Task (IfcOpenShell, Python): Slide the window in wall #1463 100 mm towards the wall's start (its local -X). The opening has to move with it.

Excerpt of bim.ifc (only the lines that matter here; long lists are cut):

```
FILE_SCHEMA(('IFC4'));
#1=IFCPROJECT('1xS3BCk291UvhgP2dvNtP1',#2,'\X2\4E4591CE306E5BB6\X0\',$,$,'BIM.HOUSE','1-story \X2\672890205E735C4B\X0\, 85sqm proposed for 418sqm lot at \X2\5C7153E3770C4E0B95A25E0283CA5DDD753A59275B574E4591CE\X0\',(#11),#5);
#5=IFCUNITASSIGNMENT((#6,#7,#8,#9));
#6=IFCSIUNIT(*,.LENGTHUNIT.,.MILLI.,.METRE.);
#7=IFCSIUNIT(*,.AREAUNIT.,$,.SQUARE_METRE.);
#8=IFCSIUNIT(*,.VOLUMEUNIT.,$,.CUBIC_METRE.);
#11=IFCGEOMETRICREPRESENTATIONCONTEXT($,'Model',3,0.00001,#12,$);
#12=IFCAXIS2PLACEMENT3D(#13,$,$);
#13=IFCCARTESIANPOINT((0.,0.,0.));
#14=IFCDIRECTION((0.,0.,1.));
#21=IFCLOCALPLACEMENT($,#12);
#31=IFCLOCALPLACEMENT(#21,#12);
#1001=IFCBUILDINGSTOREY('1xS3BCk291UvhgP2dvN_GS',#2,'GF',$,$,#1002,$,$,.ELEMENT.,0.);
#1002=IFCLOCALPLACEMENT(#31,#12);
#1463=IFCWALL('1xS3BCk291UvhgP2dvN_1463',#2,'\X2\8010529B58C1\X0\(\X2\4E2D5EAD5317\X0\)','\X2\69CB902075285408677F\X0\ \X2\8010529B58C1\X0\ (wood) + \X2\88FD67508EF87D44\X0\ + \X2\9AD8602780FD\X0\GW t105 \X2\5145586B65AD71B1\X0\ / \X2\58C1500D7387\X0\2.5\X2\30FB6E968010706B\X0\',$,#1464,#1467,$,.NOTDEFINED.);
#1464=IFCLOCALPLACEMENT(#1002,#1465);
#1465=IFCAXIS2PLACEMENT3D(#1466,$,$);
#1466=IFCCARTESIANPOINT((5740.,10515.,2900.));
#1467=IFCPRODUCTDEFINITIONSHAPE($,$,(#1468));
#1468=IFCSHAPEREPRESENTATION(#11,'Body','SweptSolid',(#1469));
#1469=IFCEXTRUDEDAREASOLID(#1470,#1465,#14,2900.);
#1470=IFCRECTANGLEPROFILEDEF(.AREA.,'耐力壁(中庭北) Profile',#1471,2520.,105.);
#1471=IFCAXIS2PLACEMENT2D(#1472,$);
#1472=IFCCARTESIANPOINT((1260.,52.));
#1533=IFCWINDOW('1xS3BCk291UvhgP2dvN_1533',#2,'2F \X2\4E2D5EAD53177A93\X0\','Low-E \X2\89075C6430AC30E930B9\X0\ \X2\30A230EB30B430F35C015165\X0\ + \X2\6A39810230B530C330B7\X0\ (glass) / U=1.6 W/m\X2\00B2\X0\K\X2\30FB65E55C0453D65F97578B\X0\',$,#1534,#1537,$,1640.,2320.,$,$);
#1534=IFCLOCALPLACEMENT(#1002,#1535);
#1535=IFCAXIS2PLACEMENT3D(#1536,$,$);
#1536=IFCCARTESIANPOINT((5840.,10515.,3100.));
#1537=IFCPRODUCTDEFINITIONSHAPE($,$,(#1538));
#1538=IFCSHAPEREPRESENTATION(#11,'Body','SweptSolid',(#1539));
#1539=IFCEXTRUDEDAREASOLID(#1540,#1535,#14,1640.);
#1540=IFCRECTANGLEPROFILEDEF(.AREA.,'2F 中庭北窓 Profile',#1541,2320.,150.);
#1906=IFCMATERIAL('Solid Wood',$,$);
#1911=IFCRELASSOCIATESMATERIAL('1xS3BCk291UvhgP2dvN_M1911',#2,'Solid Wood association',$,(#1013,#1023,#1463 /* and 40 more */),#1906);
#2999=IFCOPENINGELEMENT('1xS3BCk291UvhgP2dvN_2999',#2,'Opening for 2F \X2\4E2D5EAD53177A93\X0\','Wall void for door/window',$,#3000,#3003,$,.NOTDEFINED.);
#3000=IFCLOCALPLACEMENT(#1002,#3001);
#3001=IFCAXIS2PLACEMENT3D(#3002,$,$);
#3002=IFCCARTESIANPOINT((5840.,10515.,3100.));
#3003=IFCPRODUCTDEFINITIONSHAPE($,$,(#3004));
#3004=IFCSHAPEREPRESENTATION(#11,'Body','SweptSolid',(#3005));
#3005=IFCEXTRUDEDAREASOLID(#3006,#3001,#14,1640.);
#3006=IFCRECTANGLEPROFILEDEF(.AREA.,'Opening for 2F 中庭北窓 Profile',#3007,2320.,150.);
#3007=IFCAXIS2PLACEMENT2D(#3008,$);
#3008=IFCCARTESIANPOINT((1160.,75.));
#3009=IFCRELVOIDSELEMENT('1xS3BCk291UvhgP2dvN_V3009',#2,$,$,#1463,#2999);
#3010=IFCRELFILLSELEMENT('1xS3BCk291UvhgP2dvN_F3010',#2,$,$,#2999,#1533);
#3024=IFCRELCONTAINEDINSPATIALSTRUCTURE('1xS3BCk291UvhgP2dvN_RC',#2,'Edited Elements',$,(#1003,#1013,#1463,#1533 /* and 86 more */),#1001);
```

```python
import ifcopenshell
import ifcopenshell.api.geometry
import ifcopenshell.util.placement

model = ifcopenshell.open("bim.ifc")

window = model.by_guid("1xS3BCk291UvhgP2dvN_1533")
opening = window.FillsVoids[0].RelatingOpeningElement
wall = opening.VoidsElements[0].RelatingBuildingElement

wall_matrix = ifcopenshell.util.placement.get_local_placement(wall.ObjectPlacement)
shift = wall_matrix[:3, 0] * -100.0
before = ifcopenshell.util.placement.get_local_placement(window.ObjectPlacement)[:3, 3].copy()

# The window is not placed relative to its opening, so move both.
for product in (opening, window):
    matrix = ifcopenshell.util.placement.get_local_placement(product.ObjectPlacement)
    matrix[:3, 3] += shift
    ifcopenshell.api.geometry.edit_object_placement(model, product=product, matrix=matrix, is_si=False)

after = ifcopenshell.util.placement.get_local_placement(window.ObjectPlacement)[:3, 3]
print("window moved by", (after - before).round(3) + 0.0)

model.write("bim-out.ifc")
```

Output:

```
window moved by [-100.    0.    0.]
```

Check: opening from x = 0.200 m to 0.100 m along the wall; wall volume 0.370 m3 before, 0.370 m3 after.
